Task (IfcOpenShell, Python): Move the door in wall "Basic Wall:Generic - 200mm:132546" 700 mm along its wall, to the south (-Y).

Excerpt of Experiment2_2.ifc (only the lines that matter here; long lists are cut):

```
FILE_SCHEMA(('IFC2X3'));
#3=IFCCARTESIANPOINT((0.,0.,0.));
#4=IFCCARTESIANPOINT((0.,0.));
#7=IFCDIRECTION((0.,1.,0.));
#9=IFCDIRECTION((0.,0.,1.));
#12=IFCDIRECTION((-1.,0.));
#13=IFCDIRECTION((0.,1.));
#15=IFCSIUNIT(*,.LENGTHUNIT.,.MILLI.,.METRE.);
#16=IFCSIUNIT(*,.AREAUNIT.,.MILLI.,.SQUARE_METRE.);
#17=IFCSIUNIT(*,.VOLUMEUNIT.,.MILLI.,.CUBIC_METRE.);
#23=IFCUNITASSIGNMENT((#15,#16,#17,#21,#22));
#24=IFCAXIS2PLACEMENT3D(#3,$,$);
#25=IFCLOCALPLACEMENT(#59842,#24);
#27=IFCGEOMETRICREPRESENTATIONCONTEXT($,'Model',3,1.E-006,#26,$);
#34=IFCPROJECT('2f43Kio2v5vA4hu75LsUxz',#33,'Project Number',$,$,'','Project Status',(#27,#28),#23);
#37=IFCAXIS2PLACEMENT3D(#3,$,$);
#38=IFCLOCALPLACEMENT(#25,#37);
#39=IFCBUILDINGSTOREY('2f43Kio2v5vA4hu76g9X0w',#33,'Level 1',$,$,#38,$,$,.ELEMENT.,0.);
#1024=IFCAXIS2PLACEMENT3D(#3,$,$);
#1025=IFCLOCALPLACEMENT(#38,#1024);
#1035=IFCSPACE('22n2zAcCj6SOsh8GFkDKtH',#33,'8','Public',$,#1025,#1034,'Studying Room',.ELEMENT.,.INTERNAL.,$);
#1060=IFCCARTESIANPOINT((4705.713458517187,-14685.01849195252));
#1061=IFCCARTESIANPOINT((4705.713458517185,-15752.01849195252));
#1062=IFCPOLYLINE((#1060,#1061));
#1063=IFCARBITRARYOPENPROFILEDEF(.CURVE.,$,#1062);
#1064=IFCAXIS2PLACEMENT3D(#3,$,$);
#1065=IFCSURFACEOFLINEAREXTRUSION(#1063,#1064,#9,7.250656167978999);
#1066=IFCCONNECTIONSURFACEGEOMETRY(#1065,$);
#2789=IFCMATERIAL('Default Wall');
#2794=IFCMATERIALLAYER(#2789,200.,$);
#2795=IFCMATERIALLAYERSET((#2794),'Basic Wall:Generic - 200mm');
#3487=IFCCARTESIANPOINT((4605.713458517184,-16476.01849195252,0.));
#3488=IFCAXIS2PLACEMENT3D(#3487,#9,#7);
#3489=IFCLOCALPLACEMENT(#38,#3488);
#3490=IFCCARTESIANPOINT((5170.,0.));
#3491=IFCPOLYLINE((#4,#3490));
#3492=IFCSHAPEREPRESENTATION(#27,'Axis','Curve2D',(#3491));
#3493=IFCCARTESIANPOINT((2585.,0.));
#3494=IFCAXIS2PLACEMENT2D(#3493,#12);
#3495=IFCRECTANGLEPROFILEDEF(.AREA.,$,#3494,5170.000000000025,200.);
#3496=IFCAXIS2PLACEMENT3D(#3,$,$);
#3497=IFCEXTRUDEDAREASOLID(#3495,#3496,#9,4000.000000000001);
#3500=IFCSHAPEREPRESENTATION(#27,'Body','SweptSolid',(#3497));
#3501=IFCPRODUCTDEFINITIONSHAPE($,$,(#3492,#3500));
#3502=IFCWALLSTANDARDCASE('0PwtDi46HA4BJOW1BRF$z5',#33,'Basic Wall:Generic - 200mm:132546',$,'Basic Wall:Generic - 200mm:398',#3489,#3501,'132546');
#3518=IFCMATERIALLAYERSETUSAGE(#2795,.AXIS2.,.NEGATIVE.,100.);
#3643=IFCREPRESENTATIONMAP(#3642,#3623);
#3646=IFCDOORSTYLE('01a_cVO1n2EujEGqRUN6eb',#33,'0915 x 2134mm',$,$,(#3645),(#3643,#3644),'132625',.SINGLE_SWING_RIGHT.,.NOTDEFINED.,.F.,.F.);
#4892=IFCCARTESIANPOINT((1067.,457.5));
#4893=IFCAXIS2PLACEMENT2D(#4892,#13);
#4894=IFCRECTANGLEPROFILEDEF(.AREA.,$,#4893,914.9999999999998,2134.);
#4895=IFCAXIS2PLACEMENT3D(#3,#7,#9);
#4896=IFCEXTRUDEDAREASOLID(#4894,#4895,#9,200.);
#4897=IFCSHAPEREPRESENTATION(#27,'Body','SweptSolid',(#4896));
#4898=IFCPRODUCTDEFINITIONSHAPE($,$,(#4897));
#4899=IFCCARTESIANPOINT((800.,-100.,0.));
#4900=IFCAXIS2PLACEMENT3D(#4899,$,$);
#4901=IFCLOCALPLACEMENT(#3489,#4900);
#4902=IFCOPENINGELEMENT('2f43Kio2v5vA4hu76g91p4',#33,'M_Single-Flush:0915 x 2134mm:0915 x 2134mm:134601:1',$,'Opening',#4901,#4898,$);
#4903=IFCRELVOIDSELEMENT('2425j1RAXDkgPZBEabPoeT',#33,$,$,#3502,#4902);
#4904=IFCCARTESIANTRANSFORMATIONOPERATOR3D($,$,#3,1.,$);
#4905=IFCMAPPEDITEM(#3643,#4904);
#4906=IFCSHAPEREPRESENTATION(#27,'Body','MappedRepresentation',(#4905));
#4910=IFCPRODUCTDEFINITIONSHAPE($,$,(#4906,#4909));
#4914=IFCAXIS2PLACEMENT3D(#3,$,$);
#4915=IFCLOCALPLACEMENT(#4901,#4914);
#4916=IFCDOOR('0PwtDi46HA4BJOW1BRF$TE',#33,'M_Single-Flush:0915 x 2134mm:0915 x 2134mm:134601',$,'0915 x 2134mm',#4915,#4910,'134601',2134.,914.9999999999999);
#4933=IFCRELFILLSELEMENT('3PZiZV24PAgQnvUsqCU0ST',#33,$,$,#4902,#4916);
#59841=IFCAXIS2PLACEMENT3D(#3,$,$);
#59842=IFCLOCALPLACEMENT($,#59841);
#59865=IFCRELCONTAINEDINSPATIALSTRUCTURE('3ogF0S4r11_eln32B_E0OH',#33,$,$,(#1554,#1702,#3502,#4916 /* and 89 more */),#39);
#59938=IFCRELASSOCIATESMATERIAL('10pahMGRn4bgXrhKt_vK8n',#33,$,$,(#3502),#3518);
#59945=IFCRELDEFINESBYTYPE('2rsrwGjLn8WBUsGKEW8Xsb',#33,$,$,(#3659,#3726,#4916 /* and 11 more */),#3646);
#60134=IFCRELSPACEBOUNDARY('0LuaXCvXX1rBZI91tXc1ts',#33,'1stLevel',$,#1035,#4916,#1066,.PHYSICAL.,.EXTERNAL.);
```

```python
import numpy as np
import ifcopenshell
import ifcopenshell.api.geometry
import ifcopenshell.util.placement

model = ifcopenshell.open("Experiment2_2.ifc")

door = model.by_guid("0PwtDi46HA4BJOW1BRF$TE")
opening = door.FillsVoids[0].RelatingOpeningElement
wall = opening.VoidsElements[0].RelatingBuildingElement

wall_matrix = ifcopenshell.util.placement.get_local_placement(wall.ObjectPlacement)
shift = wall_matrix[:3, 0] * -700.0
before = ifcopenshell.util.placement.get_local_placement(door.ObjectPlacement)[:3, 3].copy()

# The door is placed relative to its opening, so it follows when the opening moves.
matrix = ifcopenshell.util.placement.get_local_placement(opening.ObjectPlacement)
matrix[:3, 3] += shift
ifcopenshell.api.geometry.edit_object_placement(
    model, product=opening, matrix=matrix, is_si=False, should_transform_children=True
)

# Space boundary surfaces are stored in each space's coordinates; move them too.
for rel in door.ProvidesBoundaries:
    if not rel.ConnectionGeometry:
        continue
    surface = rel.ConnectionGeometry.SurfaceOnRelatingElement
    space_matrix = ifcopenshell.util.placement.get_local_placement(rel.RelatingSpace.ObjectPlacement)
    point = np.array(surface.Position.Location.Coordinates) + space_matrix[:3, :3].T @ shift
    surface.Position = model.createIfcAxis2Placement3D(
        model.createIfcCartesianPoint(point.tolist()), surface.Position.Axis, surface.Position.RefDirection
    )

after = ifcopenshell.util.placement.get_local_placement(door.ObjectPlacement)[:3, 3]
print("door moved by", (after - before).round(3) + 0.0)

model.write("Experiment2_2_updated.ifc")
```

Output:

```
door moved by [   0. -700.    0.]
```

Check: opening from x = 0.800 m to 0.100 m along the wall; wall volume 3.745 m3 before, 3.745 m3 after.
